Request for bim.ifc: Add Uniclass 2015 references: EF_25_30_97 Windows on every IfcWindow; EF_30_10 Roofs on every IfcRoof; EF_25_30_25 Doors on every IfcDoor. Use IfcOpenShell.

First a look at what the model holds.

```python
import ifcopenshell

model = ifcopenshell.open("bim.ifc")
print(model.schema)
print("classifications:", [c.Name for c in model.by_type("IfcClassification")])
for ifc_class in ("IfcDoor", "IfcRoof", "IfcStair", "IfcWall", "IfcWindow"):
    print(ifc_class, len(model.by_type(ifc_class)))
```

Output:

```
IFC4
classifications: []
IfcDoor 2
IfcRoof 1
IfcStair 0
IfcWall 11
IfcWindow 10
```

```python
import ifcopenshell
import ifcopenshell.api.classification

model = ifcopenshell.open("bim.ifc")

system = ifcopenshell.api.classification.add_classification(model, classification="Uniclass 2015")

codes = {
    "IfcWindow": ("EF_25_30_97", "Windows"),
    "IfcRoof": ("EF_30_10", "Roofs"),
    "IfcDoor": ("EF_25_30_25", "Doors"),
}
for ifc_class, (code, name) in codes.items():
    products = model.by_type(ifc_class)
    ifcopenshell.api.classification.add_reference(
        model, products=products, classification=system, identification=code, name=name
    )
    print(code, len(products))

model.write("bim_v2.ifc")
```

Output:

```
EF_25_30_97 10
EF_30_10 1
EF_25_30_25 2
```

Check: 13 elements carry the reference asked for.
